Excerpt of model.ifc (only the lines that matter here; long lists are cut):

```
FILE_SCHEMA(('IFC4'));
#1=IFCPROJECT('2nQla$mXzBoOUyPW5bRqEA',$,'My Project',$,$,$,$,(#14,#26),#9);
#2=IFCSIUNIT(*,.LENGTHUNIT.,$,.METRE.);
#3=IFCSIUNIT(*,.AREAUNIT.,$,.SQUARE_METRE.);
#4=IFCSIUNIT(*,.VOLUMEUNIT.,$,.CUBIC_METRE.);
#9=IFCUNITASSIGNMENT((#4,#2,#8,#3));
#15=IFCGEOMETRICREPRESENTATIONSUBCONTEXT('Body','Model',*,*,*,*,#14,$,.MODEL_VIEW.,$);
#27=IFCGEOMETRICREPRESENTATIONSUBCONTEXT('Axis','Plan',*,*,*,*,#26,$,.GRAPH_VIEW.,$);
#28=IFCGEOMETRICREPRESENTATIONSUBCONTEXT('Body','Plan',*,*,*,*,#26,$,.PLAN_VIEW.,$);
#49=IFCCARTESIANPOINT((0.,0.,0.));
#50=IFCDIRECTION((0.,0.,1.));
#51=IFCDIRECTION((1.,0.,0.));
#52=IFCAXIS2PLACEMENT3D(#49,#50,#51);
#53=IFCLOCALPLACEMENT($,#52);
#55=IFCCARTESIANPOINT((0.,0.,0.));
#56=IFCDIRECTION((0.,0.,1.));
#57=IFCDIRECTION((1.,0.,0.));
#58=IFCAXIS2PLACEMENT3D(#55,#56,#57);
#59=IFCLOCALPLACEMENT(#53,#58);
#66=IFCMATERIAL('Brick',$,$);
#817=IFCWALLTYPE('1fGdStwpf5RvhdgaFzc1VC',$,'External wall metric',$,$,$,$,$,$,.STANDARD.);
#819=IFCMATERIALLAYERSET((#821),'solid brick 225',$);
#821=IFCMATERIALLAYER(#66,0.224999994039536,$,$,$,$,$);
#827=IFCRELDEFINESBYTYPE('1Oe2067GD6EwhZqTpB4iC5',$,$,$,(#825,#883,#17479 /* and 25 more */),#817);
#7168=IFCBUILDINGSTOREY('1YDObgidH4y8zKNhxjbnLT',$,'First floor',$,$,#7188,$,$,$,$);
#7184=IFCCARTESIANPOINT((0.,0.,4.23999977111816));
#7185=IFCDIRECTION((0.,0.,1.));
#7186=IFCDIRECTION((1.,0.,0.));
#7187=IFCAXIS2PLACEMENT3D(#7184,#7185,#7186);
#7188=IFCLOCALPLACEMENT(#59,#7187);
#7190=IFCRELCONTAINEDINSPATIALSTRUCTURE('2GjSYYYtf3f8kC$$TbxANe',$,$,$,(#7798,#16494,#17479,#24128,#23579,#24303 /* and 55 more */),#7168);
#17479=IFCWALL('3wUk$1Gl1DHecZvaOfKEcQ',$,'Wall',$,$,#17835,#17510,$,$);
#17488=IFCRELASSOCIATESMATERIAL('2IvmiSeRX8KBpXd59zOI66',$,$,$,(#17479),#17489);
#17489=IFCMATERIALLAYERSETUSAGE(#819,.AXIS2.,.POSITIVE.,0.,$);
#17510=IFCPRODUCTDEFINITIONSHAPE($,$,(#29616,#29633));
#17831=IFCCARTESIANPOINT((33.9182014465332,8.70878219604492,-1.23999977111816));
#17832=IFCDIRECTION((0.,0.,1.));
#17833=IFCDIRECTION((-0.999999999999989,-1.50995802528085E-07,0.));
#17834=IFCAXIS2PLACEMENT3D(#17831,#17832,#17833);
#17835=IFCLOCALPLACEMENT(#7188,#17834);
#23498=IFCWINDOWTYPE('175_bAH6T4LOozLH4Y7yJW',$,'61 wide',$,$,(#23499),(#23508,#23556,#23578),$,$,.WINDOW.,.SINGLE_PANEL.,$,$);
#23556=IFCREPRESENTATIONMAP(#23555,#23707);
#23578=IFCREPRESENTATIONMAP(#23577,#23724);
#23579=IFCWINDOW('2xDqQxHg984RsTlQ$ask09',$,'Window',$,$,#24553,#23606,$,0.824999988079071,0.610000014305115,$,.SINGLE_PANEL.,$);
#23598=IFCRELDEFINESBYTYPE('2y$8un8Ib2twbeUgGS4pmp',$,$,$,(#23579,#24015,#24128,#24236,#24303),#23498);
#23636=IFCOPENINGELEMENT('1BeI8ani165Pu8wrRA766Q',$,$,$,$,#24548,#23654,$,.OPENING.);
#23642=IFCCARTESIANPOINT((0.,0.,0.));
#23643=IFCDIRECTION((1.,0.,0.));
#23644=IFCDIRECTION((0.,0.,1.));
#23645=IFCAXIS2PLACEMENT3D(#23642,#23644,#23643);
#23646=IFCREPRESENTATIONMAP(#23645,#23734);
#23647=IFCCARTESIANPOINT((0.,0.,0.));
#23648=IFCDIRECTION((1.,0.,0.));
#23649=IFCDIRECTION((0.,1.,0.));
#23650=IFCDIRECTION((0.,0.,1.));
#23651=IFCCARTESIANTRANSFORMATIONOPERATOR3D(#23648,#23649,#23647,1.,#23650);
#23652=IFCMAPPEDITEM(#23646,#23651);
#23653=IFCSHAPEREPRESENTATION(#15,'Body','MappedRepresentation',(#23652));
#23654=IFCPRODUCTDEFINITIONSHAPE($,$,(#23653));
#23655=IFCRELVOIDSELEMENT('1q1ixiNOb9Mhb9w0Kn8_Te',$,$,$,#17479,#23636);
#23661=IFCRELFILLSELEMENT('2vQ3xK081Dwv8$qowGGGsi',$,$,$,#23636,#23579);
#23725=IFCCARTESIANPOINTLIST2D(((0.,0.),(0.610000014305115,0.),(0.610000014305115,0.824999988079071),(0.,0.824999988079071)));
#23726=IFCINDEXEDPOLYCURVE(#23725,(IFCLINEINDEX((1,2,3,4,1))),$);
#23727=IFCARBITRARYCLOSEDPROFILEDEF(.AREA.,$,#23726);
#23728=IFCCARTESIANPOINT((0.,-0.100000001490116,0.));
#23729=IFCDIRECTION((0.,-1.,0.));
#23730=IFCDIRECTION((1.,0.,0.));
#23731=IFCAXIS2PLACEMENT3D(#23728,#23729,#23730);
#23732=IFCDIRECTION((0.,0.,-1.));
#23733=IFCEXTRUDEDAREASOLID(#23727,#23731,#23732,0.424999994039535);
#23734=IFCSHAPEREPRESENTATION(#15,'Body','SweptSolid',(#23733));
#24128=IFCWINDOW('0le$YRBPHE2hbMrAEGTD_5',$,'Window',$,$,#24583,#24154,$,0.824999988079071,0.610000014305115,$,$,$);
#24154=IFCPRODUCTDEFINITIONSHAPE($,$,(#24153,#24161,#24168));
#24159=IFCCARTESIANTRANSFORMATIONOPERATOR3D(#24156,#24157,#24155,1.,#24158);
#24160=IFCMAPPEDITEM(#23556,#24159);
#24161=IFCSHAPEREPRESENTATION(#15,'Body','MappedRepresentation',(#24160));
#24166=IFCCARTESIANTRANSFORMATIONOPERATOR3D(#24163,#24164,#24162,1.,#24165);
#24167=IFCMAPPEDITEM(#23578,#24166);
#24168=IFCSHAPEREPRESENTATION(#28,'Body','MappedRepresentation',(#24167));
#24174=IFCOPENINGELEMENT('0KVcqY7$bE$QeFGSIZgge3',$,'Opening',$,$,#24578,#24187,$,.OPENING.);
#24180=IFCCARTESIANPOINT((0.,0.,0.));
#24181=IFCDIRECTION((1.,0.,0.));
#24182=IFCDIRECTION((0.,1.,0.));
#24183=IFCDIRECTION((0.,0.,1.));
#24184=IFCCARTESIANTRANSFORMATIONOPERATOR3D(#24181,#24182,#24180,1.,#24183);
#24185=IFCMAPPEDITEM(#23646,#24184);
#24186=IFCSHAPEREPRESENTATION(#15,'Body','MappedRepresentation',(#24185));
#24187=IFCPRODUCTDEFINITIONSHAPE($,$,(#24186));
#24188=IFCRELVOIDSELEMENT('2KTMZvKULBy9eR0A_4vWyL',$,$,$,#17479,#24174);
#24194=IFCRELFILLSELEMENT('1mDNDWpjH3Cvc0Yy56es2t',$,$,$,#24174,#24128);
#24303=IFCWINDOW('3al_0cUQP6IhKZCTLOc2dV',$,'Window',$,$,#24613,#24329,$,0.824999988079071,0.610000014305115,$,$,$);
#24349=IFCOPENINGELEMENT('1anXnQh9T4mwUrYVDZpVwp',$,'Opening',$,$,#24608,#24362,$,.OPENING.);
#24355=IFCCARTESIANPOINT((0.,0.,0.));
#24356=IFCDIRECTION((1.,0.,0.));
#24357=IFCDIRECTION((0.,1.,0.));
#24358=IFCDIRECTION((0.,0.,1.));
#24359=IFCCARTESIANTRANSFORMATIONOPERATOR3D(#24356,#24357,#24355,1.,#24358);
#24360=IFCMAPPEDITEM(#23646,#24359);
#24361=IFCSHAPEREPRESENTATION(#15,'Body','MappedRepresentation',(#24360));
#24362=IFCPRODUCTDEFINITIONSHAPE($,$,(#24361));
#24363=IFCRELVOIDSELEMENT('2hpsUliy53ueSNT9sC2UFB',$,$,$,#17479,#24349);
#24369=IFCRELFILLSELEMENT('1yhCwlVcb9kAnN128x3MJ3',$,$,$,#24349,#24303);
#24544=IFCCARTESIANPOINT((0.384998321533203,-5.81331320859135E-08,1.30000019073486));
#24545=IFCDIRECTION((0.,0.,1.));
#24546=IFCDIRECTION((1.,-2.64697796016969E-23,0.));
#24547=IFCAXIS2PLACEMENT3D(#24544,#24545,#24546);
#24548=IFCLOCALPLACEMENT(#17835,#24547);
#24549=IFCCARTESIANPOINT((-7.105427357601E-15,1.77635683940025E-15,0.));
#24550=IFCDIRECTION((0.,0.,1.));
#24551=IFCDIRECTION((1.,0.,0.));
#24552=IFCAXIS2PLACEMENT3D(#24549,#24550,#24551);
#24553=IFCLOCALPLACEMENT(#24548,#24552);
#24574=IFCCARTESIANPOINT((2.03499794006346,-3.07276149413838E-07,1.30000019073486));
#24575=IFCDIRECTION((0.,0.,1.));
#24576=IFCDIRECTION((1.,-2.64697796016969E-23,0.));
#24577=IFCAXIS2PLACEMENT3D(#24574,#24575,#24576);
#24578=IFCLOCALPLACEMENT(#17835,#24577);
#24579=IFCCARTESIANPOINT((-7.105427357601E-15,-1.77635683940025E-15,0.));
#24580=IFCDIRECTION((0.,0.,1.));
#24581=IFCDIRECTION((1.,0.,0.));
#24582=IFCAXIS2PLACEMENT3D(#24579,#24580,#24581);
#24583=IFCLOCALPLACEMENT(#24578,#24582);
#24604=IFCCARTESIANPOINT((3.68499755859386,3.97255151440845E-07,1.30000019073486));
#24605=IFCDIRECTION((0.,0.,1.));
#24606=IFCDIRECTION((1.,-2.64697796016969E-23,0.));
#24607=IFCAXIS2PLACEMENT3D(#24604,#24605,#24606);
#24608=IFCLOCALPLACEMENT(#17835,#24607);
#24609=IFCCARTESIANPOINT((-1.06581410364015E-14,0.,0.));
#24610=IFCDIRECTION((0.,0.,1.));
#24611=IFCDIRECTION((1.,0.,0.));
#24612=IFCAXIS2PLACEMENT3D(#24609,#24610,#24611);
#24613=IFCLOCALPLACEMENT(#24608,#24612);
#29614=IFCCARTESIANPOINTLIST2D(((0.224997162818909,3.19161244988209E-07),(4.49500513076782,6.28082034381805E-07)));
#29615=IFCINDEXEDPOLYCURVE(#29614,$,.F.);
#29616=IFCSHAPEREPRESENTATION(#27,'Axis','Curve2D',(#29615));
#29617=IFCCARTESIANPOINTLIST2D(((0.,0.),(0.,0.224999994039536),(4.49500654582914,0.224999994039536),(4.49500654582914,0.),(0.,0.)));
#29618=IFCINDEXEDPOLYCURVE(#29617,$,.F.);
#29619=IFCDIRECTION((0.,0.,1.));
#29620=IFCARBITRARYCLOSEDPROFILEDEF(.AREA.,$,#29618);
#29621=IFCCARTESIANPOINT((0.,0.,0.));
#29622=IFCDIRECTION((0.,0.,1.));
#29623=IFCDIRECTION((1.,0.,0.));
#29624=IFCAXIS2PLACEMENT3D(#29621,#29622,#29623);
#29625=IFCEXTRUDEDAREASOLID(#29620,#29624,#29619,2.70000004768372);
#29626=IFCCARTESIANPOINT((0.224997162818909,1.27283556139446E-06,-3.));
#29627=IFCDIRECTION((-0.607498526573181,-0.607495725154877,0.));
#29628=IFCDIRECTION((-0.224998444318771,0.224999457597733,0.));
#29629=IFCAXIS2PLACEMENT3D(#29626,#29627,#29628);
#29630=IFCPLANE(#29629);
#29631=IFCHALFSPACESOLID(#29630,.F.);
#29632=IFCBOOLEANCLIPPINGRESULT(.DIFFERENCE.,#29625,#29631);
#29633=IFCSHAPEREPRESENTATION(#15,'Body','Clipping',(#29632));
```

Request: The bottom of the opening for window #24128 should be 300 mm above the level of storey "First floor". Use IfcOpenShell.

```python
import numpy as np
import ifcopenshell
import ifcopenshell.api.geometry
import ifcopenshell.geom
import ifcopenshell.util.element
import ifcopenshell.util.placement
import ifcopenshell.util.shape
import ifcopenshell.util.unit

model = ifcopenshell.open("model.ifc")
unit_scale = ifcopenshell.util.unit.calculate_unit_scale(model)

window = model.by_guid("0le$YRBPHE2hbMrAEGTD_5")
opening = window.FillsVoids[0].RelatingOpeningElement
storey = ifcopenshell.util.element.get_container(window, ifc_class="IfcBuildingStorey")
level = ifcopenshell.util.placement.get_local_placement(storey.ObjectPlacement)[2, 3]

# The opening's origin need not be at the sill, so measure its lowest point.
shape = ifcopenshell.geom.create_shape(ifcopenshell.geom.settings(), opening)
bottom = ifcopenshell.util.shape.get_shape_bottom_elevation(shape, shape.geometry) / unit_scale
dz = level + 0.3 - bottom

shift = np.array([0.0, 0.0, dz])
# The window is placed relative to its opening, so it follows when the opening moves.
matrix = ifcopenshell.util.placement.get_local_placement(opening.ObjectPlacement)
matrix[:3, 3] += shift
ifcopenshell.api.geometry.edit_object_placement(
    model, product=opening, matrix=matrix, is_si=False, should_transform_children=True
)

print(f"moved by {dz * unit_scale:+.3f} m")

model.write("model_updated.ifc")
```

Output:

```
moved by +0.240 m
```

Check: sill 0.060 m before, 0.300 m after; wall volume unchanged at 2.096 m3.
